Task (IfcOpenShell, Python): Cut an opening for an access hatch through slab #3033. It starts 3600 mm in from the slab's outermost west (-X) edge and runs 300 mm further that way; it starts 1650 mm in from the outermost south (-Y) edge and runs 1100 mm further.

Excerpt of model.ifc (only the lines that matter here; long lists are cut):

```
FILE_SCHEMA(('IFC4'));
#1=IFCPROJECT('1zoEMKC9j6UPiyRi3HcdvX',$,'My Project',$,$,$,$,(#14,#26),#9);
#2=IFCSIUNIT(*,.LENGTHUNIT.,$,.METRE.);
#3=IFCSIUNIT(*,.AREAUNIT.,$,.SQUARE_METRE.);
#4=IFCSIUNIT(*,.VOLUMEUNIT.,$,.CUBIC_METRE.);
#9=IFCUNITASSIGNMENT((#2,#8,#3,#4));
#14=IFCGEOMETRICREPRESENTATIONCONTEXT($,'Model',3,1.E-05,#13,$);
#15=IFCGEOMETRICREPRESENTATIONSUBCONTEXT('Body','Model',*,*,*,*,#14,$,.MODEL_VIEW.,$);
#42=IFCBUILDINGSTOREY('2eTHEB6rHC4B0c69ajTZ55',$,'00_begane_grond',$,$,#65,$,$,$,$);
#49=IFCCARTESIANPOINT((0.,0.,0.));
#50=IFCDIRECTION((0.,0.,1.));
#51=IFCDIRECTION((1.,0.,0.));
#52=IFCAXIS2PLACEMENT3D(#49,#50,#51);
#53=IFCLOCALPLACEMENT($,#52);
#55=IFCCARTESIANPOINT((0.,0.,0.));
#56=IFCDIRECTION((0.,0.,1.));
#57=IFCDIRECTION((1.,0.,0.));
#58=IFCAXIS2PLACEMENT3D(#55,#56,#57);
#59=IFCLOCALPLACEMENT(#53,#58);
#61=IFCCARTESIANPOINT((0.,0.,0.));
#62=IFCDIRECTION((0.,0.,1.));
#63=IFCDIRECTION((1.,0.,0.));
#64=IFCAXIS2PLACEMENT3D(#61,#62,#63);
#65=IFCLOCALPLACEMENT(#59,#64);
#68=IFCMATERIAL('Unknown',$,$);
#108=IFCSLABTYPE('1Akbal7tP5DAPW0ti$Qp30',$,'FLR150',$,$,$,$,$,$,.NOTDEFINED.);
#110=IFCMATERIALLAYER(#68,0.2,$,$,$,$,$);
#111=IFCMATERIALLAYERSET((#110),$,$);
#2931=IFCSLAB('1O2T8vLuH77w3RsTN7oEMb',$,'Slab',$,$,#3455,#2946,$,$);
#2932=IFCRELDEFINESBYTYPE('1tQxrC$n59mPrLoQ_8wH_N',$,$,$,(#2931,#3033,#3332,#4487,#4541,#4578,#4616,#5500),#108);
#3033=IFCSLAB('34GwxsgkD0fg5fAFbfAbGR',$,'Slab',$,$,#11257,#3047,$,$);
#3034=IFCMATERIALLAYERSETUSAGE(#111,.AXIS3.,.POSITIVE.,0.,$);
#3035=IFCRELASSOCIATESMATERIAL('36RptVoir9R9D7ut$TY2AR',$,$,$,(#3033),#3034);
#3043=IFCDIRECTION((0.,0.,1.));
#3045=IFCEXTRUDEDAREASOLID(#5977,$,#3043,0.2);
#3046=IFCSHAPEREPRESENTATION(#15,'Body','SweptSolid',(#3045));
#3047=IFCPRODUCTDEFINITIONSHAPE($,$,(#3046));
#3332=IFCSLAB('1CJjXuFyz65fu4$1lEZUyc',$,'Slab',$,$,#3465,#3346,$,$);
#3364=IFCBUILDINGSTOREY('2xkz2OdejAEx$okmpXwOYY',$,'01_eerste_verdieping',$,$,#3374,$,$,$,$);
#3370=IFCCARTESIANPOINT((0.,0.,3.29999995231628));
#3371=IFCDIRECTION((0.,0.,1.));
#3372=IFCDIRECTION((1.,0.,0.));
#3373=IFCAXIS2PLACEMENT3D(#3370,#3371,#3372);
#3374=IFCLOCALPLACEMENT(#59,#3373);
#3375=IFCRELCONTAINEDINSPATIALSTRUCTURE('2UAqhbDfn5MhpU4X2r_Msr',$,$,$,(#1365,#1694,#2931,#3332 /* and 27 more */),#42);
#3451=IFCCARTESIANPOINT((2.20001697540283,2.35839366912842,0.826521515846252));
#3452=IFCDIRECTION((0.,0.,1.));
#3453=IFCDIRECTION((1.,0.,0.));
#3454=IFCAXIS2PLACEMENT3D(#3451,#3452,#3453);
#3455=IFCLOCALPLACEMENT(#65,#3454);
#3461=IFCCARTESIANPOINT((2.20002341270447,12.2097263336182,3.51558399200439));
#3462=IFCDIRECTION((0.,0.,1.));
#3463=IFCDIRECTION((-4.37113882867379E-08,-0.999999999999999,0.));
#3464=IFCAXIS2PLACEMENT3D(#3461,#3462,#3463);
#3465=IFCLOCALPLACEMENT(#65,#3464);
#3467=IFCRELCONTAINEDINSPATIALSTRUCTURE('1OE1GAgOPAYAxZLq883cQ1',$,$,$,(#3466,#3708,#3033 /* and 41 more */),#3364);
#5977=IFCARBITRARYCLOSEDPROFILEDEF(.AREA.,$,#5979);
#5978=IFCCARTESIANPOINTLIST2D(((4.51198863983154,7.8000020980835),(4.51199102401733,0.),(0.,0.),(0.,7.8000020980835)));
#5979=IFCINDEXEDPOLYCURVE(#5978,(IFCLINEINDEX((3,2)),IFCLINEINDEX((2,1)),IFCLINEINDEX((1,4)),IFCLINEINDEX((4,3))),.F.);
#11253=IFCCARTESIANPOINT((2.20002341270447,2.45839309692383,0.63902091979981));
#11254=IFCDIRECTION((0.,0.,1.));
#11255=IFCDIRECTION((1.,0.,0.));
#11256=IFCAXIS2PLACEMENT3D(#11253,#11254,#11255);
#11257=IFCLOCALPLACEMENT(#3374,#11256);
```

```python
import numpy as np
import ifcopenshell
import ifcopenshell.api.feature
import ifcopenshell.api.geometry
import ifcopenshell.api.root
import ifcopenshell.geom
import ifcopenshell.util.placement
import ifcopenshell.util.representation
import ifcopenshell.util.shape
import ifcopenshell.util.unit

model = ifcopenshell.open("model.ifc")
unit_scale = ifcopenshell.util.unit.calculate_unit_scale(model)
settings = ifcopenshell.geom.settings()


def volume(element):
    """Net volume in cubic metres, openings subtracted."""
    shape = ifcopenshell.geom.create_shape(settings, element)
    return ifcopenshell.util.shape.get_volume(shape.geometry)


slab = model.by_guid("34GwxsgkD0fg5fAFbfAbGR")
before = volume(slab)

# Extent in the slab's own axes, in metres. The edges named are its -X and -Y sides.
slab_shape = ifcopenshell.geom.create_shape(settings, slab)
vertices = ifcopenshell.util.shape.get_vertices(slab_shape.geometry)
x_min, y_min, bottom = vertices.min(axis=0)
top = vertices[:, 2].max()

opening = ifcopenshell.api.root.create_entity(model, ifc_class="IfcOpeningElement", name="Access hatch opening", predefined_type="OPENING")
context = ifcopenshell.util.representation.get_context(model, "Model", "Body", "MODEL_VIEW")
width, depth = 0.3, 1.1
outline = [(0.0, 0.0), (width, 0.0), (width, depth), (0.0, depth), (0.0, 0.0)]
# Overshoot both faces by 50 mm so the cut is clean.
shape = ifcopenshell.api.geometry.add_slab_representation(
    model, context=context, depth=top - bottom + 0.1, polyline=outline
)
ifcopenshell.api.geometry.assign_representation(model, product=opening, representation=shape)

matrix = ifcopenshell.util.placement.get_local_placement(slab.ObjectPlacement)
matrix[:, 3] = matrix @ np.append(np.array([x_min + 3.6, y_min + 1.65, bottom - 0.05]) / unit_scale, 1.0)
ifcopenshell.api.geometry.edit_object_placement(model, product=opening, matrix=matrix, is_si=False)
ifcopenshell.api.feature.add_feature(model, feature=opening, element=slab)

after = volume(slab)

print(f"slab volume {before:.3f} -> {after:.3f} m3")

model.write("model_updated.ifc")
```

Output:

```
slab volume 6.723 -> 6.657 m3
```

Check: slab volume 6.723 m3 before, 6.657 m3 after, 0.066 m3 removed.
